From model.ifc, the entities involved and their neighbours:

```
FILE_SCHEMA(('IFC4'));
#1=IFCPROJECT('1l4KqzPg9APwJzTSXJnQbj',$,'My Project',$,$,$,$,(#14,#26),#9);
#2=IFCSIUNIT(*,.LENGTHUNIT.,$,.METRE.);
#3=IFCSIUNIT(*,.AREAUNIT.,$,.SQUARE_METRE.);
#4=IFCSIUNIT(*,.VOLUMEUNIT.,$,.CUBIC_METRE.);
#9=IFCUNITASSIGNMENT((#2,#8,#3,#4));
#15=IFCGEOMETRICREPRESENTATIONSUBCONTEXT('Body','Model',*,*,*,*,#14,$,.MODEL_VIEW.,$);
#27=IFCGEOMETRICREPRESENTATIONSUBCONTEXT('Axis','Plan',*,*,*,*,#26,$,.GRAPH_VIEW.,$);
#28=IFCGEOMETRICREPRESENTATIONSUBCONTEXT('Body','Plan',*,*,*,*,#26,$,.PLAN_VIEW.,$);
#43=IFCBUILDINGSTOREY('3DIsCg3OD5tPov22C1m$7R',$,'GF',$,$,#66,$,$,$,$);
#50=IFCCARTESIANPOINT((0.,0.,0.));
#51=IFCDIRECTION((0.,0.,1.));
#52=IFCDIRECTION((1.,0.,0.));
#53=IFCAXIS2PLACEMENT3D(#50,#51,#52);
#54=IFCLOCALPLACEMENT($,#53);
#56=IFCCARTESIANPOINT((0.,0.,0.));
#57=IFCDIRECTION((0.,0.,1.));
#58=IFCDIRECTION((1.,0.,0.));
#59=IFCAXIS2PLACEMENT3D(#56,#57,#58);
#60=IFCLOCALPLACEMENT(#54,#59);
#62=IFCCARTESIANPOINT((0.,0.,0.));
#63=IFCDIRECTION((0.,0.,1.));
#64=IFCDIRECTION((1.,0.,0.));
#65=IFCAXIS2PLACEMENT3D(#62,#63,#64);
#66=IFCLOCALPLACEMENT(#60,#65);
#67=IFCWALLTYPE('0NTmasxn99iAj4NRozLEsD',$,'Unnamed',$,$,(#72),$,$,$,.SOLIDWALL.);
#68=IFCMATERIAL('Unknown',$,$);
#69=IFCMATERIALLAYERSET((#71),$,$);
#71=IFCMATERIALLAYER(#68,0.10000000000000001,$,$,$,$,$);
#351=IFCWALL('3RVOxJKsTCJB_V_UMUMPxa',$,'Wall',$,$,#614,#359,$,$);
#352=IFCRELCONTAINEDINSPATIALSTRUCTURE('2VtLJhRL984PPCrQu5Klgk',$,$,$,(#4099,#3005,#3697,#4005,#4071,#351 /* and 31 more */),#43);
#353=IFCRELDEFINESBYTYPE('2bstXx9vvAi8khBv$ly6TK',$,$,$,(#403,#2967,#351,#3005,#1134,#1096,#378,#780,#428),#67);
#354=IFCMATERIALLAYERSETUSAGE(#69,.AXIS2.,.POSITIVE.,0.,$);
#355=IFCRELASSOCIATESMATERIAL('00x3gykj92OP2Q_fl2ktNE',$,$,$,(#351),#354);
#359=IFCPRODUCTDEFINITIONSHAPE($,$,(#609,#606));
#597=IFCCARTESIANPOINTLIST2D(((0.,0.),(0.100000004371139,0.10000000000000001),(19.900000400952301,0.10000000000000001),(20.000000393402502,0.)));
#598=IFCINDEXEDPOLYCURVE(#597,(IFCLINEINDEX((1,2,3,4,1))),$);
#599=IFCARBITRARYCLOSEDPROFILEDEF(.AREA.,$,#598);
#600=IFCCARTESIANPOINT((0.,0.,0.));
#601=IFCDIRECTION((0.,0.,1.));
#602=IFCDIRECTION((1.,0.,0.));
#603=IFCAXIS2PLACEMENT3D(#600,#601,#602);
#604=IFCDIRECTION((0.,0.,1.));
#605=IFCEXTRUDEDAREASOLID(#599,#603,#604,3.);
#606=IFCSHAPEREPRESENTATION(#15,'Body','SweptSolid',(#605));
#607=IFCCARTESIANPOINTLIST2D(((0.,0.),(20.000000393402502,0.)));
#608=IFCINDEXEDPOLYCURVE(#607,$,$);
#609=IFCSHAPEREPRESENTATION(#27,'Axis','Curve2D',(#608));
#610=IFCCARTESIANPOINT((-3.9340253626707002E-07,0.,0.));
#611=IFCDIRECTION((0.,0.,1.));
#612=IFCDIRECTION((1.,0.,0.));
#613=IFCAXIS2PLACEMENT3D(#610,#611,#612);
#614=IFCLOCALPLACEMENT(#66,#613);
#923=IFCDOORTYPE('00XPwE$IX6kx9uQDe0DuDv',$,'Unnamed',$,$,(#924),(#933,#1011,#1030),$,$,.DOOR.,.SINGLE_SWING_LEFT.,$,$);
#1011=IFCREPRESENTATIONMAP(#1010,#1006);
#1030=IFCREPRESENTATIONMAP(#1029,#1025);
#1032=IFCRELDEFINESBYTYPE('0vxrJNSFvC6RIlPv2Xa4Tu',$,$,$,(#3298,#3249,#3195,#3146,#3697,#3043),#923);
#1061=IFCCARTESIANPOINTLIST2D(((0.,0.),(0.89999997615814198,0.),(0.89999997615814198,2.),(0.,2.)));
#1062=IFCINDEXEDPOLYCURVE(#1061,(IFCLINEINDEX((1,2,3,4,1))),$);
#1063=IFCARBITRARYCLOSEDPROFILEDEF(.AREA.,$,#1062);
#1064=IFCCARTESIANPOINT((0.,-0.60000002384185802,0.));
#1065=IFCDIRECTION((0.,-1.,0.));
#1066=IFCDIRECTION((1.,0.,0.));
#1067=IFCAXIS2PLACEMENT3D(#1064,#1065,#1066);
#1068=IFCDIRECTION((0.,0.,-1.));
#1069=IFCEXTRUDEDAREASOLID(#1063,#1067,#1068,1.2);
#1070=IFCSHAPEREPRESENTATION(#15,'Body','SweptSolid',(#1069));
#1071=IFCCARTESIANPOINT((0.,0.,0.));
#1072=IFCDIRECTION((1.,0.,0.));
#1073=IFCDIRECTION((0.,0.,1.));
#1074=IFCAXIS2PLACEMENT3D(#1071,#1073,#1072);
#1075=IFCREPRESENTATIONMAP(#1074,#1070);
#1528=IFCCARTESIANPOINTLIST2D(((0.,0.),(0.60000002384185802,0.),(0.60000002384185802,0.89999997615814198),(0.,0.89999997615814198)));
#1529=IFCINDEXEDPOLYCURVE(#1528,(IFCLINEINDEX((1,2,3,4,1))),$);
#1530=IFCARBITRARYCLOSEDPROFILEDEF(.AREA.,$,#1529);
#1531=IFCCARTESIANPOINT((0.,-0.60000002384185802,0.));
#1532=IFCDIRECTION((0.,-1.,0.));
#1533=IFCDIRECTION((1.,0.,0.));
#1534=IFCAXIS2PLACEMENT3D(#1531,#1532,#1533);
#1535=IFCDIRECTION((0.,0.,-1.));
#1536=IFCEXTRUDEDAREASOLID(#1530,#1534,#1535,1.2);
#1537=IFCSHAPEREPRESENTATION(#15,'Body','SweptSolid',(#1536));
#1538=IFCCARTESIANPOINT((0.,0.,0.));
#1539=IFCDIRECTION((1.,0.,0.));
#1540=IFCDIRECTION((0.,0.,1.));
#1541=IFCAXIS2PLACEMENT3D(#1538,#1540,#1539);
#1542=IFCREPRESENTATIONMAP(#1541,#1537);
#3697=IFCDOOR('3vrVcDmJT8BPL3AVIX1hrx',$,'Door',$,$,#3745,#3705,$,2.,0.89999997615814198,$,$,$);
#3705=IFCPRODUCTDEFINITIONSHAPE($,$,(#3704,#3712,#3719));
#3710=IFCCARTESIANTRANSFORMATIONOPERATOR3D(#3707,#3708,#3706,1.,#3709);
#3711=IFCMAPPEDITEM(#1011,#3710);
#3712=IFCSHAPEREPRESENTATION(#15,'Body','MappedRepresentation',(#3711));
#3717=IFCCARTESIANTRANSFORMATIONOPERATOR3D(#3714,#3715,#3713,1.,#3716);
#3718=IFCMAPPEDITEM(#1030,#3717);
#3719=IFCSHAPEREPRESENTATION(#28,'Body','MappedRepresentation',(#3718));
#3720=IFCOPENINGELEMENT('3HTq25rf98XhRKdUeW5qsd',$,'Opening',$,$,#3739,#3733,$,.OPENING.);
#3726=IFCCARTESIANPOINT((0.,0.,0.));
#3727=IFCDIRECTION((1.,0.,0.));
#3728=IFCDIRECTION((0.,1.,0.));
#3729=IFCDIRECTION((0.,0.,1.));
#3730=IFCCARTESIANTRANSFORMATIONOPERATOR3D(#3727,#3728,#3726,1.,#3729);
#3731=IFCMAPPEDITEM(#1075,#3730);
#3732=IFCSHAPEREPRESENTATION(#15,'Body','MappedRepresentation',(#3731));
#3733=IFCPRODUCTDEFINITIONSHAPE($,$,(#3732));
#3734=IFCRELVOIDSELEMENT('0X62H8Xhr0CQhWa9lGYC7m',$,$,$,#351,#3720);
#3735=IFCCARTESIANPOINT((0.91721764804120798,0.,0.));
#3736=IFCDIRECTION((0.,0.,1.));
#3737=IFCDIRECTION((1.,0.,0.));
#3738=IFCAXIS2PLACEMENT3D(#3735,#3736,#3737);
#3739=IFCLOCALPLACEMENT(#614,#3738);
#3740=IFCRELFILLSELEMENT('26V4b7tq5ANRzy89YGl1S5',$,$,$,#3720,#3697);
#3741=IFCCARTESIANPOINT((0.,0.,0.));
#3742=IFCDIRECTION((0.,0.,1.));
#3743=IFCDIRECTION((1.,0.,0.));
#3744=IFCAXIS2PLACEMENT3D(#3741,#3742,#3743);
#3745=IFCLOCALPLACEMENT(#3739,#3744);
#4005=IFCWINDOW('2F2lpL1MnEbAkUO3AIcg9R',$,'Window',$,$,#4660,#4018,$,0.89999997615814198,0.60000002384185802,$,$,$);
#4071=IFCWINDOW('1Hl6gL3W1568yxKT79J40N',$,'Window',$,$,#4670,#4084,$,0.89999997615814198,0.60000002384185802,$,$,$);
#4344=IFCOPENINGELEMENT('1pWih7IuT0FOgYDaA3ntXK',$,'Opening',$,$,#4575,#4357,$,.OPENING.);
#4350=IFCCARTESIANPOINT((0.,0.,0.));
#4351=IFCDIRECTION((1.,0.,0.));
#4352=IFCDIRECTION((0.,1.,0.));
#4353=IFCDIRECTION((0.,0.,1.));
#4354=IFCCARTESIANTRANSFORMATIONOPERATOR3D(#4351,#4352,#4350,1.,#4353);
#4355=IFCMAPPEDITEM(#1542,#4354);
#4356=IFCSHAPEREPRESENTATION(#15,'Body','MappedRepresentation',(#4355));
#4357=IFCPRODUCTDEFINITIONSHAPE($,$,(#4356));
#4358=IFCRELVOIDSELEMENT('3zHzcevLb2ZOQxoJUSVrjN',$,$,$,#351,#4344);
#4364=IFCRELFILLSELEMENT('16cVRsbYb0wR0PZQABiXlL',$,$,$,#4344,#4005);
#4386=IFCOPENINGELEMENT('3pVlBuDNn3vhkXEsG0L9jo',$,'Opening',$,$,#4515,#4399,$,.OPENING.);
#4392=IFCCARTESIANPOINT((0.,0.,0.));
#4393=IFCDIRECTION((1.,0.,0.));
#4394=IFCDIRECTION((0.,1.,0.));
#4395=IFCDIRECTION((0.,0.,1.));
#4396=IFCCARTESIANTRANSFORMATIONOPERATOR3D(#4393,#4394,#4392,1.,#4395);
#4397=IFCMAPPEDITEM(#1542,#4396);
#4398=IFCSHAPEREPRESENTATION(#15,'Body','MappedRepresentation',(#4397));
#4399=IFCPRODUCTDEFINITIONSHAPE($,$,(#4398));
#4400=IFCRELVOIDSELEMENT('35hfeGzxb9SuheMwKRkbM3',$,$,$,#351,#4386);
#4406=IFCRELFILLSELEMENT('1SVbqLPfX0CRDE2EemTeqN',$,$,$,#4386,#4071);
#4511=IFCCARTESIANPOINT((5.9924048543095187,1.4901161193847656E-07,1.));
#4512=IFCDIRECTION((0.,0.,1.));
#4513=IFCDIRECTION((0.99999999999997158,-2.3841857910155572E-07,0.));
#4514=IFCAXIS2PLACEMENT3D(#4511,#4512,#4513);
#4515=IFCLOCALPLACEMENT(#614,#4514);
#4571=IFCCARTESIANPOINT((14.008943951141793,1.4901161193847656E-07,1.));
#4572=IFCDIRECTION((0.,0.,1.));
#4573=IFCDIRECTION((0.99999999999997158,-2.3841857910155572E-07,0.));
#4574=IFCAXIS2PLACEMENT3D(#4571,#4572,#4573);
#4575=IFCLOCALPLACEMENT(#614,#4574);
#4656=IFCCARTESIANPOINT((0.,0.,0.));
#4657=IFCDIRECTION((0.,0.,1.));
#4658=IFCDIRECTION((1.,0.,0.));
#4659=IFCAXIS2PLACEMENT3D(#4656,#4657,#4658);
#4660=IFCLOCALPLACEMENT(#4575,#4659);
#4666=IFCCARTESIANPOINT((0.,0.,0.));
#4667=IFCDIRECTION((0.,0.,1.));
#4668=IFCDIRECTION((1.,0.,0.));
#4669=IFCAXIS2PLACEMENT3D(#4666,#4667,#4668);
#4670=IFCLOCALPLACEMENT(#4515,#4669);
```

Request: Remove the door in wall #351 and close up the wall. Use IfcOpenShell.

```python
import ifcopenshell
import ifcopenshell.api.feature
import ifcopenshell.api.root
import ifcopenshell.geom
import ifcopenshell.util.shape

model = ifcopenshell.open("model.ifc")
settings = ifcopenshell.geom.settings()


def volume(element):
    """Net volume in cubic metres, openings subtracted."""
    shape = ifcopenshell.geom.create_shape(settings, element)
    return ifcopenshell.util.shape.get_volume(shape.geometry)


door = model.by_guid("3vrVcDmJT8BPL3AVIX1hrx")
opening = door.FillsVoids[0].RelatingOpeningElement
wall = opening.VoidsElements[0].RelatingBuildingElement
before = volume(wall)

ifcopenshell.api.root.remove_product(model, product=door)
ifcopenshell.api.feature.remove_feature(model, feature=opening)

after = volume(wall)

print(f"wall volume {before:.3f} -> {after:.3f} m3")

model.write("model_updated.ifc")
```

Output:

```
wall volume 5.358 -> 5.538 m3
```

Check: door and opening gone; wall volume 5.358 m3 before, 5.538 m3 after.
